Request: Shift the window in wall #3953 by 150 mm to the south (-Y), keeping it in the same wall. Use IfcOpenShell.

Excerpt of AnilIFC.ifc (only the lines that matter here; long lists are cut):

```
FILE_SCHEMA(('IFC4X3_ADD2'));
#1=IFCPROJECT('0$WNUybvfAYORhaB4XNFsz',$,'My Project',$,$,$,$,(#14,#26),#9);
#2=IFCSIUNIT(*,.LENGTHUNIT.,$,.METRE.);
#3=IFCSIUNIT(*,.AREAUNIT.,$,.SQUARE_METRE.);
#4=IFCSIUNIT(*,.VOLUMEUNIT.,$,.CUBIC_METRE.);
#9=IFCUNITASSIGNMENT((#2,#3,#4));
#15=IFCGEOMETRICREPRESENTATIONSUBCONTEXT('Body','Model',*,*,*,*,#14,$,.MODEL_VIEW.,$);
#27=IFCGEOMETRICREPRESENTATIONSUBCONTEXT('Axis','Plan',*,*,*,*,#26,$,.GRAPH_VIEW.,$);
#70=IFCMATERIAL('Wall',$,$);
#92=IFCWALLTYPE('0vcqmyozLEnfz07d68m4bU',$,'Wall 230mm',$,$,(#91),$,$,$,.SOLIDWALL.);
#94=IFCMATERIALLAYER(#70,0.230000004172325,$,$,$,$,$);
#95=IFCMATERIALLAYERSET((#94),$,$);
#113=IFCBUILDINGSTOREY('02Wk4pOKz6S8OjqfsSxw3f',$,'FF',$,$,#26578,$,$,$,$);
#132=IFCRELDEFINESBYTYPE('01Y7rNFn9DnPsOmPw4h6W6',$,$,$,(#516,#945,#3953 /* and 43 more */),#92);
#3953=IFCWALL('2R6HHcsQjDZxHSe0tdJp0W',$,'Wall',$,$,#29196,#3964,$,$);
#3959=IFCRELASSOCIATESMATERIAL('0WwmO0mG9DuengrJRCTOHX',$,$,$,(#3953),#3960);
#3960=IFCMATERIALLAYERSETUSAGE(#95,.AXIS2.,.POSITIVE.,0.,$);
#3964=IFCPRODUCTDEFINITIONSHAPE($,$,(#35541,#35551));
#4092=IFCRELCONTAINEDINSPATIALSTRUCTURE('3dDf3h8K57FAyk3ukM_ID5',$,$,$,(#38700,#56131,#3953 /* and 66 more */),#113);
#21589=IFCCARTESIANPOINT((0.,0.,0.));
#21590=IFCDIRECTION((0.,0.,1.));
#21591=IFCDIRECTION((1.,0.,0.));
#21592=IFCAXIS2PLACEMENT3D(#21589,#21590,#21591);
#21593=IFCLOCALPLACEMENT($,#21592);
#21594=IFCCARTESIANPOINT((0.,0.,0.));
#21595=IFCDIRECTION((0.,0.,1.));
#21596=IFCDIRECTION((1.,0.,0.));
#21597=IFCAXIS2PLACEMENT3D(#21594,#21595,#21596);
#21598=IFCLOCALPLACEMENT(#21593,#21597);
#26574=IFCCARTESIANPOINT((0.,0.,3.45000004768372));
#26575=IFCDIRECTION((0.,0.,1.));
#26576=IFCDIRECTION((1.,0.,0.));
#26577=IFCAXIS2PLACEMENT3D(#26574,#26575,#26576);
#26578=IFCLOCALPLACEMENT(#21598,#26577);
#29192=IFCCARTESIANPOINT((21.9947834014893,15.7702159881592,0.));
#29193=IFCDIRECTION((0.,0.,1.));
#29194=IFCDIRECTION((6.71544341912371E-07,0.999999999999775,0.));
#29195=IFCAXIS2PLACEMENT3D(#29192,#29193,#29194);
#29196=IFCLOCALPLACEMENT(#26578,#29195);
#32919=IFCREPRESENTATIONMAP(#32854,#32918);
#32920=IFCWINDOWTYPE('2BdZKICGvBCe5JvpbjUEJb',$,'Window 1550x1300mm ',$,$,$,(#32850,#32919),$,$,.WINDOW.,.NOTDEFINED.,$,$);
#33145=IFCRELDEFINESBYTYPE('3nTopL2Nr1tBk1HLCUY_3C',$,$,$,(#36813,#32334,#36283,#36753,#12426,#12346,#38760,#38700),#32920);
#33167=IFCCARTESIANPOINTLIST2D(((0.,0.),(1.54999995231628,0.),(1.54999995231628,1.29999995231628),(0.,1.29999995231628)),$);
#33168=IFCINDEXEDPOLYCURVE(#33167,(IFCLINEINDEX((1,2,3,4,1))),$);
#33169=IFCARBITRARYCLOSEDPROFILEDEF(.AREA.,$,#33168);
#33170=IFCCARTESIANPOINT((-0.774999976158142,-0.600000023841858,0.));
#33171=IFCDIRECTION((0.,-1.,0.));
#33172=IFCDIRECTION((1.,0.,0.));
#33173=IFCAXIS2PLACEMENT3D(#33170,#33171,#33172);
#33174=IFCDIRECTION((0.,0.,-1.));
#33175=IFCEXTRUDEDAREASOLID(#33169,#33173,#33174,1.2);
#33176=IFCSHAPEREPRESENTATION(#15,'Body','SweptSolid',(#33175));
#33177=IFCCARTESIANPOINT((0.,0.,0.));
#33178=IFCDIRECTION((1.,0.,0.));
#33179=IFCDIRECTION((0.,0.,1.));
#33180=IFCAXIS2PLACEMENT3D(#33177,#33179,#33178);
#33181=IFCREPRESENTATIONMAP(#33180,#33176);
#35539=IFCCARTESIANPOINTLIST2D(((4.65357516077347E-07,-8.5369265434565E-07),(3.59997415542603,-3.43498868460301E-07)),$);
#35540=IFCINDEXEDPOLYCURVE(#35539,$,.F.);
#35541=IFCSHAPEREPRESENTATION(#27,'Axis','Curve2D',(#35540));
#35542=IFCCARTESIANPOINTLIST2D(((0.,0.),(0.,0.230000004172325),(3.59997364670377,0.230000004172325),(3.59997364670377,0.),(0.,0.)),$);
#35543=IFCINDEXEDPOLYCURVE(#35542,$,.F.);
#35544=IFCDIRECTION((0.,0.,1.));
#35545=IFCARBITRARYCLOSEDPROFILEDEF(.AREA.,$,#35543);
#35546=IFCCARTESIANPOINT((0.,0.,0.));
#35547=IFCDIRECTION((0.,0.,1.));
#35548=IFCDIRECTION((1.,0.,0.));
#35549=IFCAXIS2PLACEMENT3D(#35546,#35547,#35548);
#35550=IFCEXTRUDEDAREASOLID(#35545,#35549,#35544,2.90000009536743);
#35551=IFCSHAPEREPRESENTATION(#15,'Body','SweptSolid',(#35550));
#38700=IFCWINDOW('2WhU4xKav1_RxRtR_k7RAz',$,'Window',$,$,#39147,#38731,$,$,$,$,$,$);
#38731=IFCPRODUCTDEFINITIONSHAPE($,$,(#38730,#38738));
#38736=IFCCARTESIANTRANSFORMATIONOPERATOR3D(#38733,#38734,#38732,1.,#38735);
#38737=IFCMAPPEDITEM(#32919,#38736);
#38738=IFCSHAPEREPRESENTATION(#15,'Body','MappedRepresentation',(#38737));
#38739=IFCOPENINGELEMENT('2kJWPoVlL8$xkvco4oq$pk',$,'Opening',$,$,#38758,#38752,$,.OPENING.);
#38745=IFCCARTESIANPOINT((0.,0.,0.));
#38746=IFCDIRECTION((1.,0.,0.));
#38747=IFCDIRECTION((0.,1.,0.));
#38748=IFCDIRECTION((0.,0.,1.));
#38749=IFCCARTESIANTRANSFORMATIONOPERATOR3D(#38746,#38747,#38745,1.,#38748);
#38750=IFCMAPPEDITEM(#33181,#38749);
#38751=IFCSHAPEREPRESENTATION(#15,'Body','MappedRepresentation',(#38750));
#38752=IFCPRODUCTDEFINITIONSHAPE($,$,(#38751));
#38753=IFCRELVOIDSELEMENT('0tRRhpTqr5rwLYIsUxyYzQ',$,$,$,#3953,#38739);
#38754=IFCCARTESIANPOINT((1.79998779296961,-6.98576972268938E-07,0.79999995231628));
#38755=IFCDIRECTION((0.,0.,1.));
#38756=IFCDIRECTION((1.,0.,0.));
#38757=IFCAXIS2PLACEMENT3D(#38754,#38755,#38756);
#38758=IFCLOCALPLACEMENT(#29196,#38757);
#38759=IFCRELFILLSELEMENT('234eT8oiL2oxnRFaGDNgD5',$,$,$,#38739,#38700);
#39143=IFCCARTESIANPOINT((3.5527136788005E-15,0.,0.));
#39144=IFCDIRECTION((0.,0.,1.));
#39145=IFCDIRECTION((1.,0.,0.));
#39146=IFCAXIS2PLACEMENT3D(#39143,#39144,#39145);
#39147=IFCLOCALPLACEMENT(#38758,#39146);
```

```python
import ifcopenshell
import ifcopenshell.api.geometry
import ifcopenshell.util.placement

model = ifcopenshell.open("AnilIFC.ifc")

window = model.by_id(38700)
opening = window.FillsVoids[0].RelatingOpeningElement
wall = opening.VoidsElements[0].RelatingBuildingElement

wall_matrix = ifcopenshell.util.placement.get_local_placement(wall.ObjectPlacement)
shift = wall_matrix[:3, 0] * -0.15
before = ifcopenshell.util.placement.get_local_placement(window.ObjectPlacement)[:3, 3].copy()

# The window is placed relative to its opening, so it follows when the opening moves.
matrix = ifcopenshell.util.placement.get_local_placement(opening.ObjectPlacement)
matrix[:3, 3] += shift
ifcopenshell.api.geometry.edit_object_placement(
    model, product=opening, matrix=matrix, is_si=False, should_transform_children=True
)

after = ifcopenshell.util.placement.get_local_placement(window.ObjectPlacement)[:3, 3]
print("window moved by", (after - before).round(3) + 0.0)

model.write("AnilIFC-out.ifc")
```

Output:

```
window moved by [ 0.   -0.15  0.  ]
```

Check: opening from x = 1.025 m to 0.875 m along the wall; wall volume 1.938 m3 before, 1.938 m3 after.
